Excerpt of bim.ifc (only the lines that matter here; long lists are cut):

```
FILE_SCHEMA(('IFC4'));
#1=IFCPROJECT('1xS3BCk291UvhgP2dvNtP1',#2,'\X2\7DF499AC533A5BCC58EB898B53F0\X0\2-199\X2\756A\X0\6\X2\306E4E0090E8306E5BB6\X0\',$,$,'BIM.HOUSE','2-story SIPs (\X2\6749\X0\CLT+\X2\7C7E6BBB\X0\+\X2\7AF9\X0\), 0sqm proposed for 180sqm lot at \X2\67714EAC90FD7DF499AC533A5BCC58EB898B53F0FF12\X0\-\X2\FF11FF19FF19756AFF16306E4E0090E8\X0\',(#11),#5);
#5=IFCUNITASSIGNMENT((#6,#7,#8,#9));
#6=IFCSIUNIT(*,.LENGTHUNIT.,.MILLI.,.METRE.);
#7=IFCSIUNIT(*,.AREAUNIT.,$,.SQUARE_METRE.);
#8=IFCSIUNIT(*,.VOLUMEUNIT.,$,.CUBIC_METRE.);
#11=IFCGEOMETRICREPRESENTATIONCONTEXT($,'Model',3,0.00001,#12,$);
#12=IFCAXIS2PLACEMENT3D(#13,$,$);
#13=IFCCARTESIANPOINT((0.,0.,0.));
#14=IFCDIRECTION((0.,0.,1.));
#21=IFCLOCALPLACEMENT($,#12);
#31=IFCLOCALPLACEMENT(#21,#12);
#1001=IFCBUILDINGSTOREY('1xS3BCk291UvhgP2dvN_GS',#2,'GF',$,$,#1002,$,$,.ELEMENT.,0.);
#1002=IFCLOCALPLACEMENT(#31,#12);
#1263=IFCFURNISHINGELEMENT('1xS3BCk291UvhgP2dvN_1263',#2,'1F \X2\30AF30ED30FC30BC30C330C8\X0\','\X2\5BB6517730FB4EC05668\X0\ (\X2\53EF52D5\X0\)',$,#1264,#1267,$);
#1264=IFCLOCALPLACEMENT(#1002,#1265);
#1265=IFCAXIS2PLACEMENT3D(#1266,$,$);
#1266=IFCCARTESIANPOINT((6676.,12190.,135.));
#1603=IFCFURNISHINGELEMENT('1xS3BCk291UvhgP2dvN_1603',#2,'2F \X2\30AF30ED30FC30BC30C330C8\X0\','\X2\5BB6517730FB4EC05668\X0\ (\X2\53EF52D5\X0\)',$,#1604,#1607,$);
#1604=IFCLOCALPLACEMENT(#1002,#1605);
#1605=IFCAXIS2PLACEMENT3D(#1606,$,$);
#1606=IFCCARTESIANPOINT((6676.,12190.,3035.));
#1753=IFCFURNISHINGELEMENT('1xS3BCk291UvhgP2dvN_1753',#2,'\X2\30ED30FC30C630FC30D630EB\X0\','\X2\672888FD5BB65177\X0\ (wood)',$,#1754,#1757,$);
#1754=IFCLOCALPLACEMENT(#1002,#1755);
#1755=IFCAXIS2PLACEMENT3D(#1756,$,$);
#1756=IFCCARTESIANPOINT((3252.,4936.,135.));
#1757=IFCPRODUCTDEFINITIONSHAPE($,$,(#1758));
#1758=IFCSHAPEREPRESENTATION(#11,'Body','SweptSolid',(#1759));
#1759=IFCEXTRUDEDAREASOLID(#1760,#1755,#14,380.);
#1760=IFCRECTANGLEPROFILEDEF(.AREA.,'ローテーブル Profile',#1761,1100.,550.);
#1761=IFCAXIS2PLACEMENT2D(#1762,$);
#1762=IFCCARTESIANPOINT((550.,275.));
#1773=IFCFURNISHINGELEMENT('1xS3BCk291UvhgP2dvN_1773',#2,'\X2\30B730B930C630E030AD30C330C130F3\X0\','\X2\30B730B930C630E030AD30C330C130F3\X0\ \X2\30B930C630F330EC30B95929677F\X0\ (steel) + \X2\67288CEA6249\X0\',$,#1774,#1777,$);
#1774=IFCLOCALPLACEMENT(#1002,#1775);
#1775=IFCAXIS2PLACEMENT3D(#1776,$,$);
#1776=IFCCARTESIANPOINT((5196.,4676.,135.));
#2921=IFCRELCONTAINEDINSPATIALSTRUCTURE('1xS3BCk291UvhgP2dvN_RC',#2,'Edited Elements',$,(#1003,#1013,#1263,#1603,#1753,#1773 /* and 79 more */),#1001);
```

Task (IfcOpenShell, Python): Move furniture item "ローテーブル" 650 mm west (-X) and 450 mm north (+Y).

```python
import ifcopenshell
import ifcopenshell.api.geometry
import ifcopenshell.util.placement
import ifcopenshell.util.unit

model = ifcopenshell.open("bim.ifc")
unit_scale = ifcopenshell.util.unit.calculate_unit_scale(model)

item = model.by_guid("1xS3BCk291UvhgP2dvN_1753")
matrix = ifcopenshell.util.placement.get_local_placement(item.ObjectPlacement)
matrix[0, 3] -= 0.65 / unit_scale
matrix[1, 3] += 0.45 / unit_scale
ifcopenshell.api.geometry.edit_object_placement(model, product=item, matrix=matrix, is_si=False)

print(ifcopenshell.util.placement.get_local_placement(item.ObjectPlacement).round(3) + 0.0)

model.write("bim_updated.ifc")
```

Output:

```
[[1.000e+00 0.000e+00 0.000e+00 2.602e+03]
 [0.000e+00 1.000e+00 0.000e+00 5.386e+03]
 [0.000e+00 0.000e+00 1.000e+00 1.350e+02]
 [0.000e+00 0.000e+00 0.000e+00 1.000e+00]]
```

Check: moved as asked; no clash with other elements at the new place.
